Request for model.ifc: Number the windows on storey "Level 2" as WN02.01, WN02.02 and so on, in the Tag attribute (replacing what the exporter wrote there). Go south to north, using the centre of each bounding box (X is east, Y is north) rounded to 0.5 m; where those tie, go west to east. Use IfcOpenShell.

First a look at what the model holds.

```python
import ifcopenshell
import ifcopenshell.util.element
import ifcopenshell.util.placement

model = ifcopenshell.open("model.ifc")
print(model.schema)
storey = next(s for s in model.by_type("IfcBuildingStorey") if s.Name == "Level 2")
windows = [e for e in ifcopenshell.util.element.get_decomposition(storey) if e.is_a("IfcWindow")]
for e in sorted(windows, key=lambda e: e.id()):
    origin = ifcopenshell.util.placement.get_local_placement(e.ObjectPlacement)[:3, 3]
    print(e.id(), e.Tag, e.Name, origin.round(2) + 0.0, sep=" | ")
```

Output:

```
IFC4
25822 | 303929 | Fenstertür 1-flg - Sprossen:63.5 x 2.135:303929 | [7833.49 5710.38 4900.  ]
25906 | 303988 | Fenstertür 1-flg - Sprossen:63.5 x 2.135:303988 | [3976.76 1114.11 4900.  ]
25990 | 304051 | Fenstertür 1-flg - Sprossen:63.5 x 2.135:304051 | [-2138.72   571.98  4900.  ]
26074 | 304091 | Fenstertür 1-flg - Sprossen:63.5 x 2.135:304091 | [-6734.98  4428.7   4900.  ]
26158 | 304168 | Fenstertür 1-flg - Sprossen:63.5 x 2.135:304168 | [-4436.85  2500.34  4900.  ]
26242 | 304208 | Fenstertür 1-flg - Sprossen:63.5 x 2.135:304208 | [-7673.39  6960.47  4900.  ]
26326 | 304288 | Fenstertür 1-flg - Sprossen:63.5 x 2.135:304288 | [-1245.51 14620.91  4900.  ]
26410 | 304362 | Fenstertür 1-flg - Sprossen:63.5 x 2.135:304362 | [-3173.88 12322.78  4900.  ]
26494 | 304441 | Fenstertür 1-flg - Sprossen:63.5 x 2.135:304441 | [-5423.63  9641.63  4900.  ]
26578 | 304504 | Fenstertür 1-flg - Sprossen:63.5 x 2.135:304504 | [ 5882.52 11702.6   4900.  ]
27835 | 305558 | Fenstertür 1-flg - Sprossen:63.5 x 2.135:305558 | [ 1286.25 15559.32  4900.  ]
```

```python
import ifcopenshell
import ifcopenshell.geom
import ifcopenshell.util.element
import ifcopenshell.util.shape

model = ifcopenshell.open("model.ifc")
settings = ifcopenshell.geom.settings()
settings.set("use-world-coords", True)


def centre(element):
    shape = ifcopenshell.geom.create_shape(settings, element)
    return ifcopenshell.util.shape.get_bbox_centroid(shape.geometry)


storey = next(s for s in model.by_type("IfcBuildingStorey") if s.Name == "Level 2")
windows = [e for e in ifcopenshell.util.element.get_decomposition(storey) if e.is_a("IfcWindow")]

# Insertion points can sit at a corner or the storey origin, so sort by the geometry (in metres).
centres = {e: centre(e) for e in windows}
windows.sort(key=lambda e: (round(centres[e][1] / 0.5), centres[e][0]))

for i, e in enumerate(windows, start=1):
    number = f"WN02.{i:02d}"
    e.Tag = number
    print(e.id(), number)

model.write("model_updated.ifc")
```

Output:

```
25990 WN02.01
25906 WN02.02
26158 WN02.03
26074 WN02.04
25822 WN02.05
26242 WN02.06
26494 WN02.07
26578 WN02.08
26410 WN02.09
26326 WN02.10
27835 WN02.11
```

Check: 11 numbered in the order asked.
